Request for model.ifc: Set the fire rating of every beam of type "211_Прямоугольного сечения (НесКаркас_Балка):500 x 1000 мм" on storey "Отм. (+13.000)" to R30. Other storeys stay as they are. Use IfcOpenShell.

First a look at what the model holds.

```python
import ifcopenshell
import ifcopenshell.util.element

model = ifcopenshell.open("model.ifc")
print(model.schema)
storey = next(s for s in model.by_type("IfcBuildingStorey") if s.Name == "Отм. (+13.000)")
beams = [e for e in ifcopenshell.util.element.get_decomposition(storey) if e.is_a("IfcBeam")]
seen = {}
for e in beams:
    element_type = ifcopenshell.util.element.get_type(e)
    key = (element_type.Name if element_type != e and element_type else None, ifcopenshell.util.element.get_pset(e, "Pset_BeamCommon", "FireRating"))
    seen[key] = seen.get(key, 0) + 1
for (name, value), count in sorted(seen.items(), key=str):
    print(count, "x", name, "|", value)
```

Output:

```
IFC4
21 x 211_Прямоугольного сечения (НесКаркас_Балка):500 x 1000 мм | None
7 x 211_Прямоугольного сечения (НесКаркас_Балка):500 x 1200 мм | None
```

```python
import ifcopenshell
import ifcopenshell.api.pset
import ifcopenshell.util.element

model = ifcopenshell.open("model.ifc")

storey = next(s for s in model.by_type("IfcBuildingStorey") if s.Name == "Отм. (+13.000)")
beams = [e for e in ifcopenshell.util.element.get_decomposition(storey) if e.is_a("IfcBeam")]

count = 0
for e in beams:
    element_type = ifcopenshell.util.element.get_type(e)
    if element_type in (None, e) or element_type.Name != "211_Прямоугольного сечения (НесКаркас_Балка):500 x 1000 мм":
        continue
    # add_pset returns the element's existing set when there is one.
    pset = ifcopenshell.api.pset.add_pset(model, product=e, name="Pset_BeamCommon")
    ifcopenshell.api.pset.edit_pset(model, pset=pset, properties={"FireRating": "R30"})
    count += 1

print(count, "beams updated")

model.write("model_updated.ifc")
```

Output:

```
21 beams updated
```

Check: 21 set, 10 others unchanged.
